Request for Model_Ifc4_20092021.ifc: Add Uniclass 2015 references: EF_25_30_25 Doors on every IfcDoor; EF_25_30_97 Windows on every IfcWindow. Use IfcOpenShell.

First a look at what the model holds.

```python
import ifcopenshell

model = ifcopenshell.open("Model_Ifc4_20092021.ifc")
print(model.schema)
print("classifications:", [c.Name for c in model.by_type("IfcClassification")])
for ifc_class in ("IfcDoor", "IfcRoof", "IfcStair", "IfcWall", "IfcWindow"):
    print(ifc_class, len(model.by_type(ifc_class)))
```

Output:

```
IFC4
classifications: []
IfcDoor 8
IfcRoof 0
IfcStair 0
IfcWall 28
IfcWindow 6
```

```python
import ifcopenshell
import ifcopenshell.api.classification

model = ifcopenshell.open("Model_Ifc4_20092021.ifc")

system = ifcopenshell.api.classification.add_classification(model, classification="Uniclass 2015")

codes = {
    "IfcDoor": ("EF_25_30_25", "Doors"),
    "IfcWindow": ("EF_25_30_97", "Windows"),
}
for ifc_class, (code, name) in codes.items():
    products = model.by_type(ifc_class)
    ifcopenshell.api.classification.add_reference(
        model, products=products, classification=system, identification=code, name=name
    )
    print(code, len(products))

model.write("Model_Ifc4_20092021_v2.ifc")
```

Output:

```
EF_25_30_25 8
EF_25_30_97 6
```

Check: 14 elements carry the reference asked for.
